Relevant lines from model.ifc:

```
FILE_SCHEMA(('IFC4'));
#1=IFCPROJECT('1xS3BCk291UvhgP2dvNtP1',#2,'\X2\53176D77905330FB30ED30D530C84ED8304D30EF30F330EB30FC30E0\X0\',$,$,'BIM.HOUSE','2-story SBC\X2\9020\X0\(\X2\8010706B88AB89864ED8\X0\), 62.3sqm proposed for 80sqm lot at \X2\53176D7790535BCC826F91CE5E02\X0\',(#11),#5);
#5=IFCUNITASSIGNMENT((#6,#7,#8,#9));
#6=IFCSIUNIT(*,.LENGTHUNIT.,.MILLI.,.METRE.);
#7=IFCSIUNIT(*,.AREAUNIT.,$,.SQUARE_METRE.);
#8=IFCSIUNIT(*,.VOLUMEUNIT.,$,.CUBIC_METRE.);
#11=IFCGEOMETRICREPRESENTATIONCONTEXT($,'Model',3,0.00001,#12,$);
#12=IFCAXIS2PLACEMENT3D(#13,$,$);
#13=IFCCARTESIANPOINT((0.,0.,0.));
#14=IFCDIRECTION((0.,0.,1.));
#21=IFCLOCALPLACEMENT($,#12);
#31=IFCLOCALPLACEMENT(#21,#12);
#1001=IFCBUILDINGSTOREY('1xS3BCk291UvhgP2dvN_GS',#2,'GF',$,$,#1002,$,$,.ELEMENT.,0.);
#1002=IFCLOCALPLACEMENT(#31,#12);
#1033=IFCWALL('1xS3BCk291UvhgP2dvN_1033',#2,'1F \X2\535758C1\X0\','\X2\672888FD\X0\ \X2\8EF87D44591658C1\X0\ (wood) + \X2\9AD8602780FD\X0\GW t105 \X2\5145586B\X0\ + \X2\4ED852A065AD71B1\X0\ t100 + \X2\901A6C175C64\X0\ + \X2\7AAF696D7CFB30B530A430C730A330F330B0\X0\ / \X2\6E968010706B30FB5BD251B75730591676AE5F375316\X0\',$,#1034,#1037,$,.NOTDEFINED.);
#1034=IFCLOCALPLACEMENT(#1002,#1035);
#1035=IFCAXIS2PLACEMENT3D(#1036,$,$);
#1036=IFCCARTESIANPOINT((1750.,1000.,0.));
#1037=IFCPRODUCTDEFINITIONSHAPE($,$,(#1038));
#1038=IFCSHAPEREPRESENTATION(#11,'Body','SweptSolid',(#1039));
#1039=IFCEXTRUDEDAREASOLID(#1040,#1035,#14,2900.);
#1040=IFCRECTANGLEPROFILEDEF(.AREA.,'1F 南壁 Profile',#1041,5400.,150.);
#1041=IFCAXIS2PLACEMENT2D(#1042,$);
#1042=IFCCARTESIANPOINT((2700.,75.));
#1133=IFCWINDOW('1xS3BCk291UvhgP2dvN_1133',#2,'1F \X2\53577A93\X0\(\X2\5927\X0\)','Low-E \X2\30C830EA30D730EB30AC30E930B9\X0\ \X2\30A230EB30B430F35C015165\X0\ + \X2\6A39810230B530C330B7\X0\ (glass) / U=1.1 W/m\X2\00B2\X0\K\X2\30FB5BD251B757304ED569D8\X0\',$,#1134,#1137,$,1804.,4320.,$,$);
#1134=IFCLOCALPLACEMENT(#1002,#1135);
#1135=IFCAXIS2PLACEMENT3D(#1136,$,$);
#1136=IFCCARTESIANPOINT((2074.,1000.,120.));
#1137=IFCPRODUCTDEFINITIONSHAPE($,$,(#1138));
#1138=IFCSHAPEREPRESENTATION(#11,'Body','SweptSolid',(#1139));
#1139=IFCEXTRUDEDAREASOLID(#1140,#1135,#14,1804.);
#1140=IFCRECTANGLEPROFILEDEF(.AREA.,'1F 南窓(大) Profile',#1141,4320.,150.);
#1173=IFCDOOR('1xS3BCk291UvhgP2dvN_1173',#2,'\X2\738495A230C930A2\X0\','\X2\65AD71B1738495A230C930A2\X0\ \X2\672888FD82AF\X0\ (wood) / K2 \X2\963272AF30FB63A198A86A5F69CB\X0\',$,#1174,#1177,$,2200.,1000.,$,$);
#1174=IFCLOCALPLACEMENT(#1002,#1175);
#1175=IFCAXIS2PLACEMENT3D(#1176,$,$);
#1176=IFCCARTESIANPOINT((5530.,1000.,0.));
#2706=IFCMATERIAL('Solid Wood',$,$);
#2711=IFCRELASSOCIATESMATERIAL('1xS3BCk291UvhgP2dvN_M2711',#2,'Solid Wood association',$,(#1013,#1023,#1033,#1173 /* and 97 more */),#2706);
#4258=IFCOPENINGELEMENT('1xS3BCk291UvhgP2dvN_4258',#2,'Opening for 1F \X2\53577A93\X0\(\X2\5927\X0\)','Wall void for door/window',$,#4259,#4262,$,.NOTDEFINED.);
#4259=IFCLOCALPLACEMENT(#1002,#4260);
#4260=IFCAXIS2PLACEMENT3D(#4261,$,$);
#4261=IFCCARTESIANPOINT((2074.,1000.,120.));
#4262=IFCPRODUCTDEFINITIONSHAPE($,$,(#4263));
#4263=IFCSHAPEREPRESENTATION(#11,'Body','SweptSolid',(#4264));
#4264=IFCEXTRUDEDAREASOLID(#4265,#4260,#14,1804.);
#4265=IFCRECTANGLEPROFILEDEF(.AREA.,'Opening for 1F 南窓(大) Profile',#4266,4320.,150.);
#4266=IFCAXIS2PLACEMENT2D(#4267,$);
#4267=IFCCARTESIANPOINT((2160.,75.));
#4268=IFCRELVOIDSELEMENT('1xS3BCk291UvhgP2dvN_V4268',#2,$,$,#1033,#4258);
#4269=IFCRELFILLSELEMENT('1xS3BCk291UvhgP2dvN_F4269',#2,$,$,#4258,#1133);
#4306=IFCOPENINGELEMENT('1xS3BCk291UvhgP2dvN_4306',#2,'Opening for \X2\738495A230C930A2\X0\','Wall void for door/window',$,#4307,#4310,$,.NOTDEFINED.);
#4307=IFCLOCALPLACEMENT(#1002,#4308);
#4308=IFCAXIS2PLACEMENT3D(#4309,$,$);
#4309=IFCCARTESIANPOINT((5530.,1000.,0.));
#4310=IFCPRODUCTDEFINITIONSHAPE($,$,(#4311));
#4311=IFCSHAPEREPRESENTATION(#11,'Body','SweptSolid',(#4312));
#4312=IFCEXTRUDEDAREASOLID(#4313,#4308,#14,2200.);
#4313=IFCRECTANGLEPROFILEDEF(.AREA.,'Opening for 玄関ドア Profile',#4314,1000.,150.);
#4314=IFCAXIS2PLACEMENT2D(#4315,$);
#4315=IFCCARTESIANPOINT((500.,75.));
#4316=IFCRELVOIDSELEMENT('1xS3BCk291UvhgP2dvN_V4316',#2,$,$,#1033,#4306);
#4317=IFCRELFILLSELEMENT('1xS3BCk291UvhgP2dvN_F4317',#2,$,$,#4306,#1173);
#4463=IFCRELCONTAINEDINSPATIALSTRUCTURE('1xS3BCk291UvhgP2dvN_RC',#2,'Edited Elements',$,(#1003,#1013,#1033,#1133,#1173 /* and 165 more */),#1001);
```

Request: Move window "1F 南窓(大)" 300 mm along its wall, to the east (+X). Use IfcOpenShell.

```python
import ifcopenshell
import ifcopenshell.api.geometry
import ifcopenshell.util.placement
import ifcopenshell.util.unit

model = ifcopenshell.open("model.ifc")
unit_scale = ifcopenshell.util.unit.calculate_unit_scale(model)

window = model.by_guid("1xS3BCk291UvhgP2dvN_1133")
opening = window.FillsVoids[0].RelatingOpeningElement
wall = opening.VoidsElements[0].RelatingBuildingElement

wall_matrix = ifcopenshell.util.placement.get_local_placement(wall.ObjectPlacement)
shift = wall_matrix[:3, 0] * 0.3 / unit_scale
before = ifcopenshell.util.placement.get_local_placement(window.ObjectPlacement)[:3, 3].copy()

# The window is not placed relative to its opening, so move both.
for product in (opening, window):
    matrix = ifcopenshell.util.placement.get_local_placement(product.ObjectPlacement)
    matrix[:3, 3] += shift
    ifcopenshell.api.geometry.edit_object_placement(model, product=product, matrix=matrix, is_si=False)

after = ifcopenshell.util.placement.get_local_placement(window.ObjectPlacement)[:3, 3]
print("window moved by", (after - before).round(3) + 0.0)

model.write("model_edited.ifc")
```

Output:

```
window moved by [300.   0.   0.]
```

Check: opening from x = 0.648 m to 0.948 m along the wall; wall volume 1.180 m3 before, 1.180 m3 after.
